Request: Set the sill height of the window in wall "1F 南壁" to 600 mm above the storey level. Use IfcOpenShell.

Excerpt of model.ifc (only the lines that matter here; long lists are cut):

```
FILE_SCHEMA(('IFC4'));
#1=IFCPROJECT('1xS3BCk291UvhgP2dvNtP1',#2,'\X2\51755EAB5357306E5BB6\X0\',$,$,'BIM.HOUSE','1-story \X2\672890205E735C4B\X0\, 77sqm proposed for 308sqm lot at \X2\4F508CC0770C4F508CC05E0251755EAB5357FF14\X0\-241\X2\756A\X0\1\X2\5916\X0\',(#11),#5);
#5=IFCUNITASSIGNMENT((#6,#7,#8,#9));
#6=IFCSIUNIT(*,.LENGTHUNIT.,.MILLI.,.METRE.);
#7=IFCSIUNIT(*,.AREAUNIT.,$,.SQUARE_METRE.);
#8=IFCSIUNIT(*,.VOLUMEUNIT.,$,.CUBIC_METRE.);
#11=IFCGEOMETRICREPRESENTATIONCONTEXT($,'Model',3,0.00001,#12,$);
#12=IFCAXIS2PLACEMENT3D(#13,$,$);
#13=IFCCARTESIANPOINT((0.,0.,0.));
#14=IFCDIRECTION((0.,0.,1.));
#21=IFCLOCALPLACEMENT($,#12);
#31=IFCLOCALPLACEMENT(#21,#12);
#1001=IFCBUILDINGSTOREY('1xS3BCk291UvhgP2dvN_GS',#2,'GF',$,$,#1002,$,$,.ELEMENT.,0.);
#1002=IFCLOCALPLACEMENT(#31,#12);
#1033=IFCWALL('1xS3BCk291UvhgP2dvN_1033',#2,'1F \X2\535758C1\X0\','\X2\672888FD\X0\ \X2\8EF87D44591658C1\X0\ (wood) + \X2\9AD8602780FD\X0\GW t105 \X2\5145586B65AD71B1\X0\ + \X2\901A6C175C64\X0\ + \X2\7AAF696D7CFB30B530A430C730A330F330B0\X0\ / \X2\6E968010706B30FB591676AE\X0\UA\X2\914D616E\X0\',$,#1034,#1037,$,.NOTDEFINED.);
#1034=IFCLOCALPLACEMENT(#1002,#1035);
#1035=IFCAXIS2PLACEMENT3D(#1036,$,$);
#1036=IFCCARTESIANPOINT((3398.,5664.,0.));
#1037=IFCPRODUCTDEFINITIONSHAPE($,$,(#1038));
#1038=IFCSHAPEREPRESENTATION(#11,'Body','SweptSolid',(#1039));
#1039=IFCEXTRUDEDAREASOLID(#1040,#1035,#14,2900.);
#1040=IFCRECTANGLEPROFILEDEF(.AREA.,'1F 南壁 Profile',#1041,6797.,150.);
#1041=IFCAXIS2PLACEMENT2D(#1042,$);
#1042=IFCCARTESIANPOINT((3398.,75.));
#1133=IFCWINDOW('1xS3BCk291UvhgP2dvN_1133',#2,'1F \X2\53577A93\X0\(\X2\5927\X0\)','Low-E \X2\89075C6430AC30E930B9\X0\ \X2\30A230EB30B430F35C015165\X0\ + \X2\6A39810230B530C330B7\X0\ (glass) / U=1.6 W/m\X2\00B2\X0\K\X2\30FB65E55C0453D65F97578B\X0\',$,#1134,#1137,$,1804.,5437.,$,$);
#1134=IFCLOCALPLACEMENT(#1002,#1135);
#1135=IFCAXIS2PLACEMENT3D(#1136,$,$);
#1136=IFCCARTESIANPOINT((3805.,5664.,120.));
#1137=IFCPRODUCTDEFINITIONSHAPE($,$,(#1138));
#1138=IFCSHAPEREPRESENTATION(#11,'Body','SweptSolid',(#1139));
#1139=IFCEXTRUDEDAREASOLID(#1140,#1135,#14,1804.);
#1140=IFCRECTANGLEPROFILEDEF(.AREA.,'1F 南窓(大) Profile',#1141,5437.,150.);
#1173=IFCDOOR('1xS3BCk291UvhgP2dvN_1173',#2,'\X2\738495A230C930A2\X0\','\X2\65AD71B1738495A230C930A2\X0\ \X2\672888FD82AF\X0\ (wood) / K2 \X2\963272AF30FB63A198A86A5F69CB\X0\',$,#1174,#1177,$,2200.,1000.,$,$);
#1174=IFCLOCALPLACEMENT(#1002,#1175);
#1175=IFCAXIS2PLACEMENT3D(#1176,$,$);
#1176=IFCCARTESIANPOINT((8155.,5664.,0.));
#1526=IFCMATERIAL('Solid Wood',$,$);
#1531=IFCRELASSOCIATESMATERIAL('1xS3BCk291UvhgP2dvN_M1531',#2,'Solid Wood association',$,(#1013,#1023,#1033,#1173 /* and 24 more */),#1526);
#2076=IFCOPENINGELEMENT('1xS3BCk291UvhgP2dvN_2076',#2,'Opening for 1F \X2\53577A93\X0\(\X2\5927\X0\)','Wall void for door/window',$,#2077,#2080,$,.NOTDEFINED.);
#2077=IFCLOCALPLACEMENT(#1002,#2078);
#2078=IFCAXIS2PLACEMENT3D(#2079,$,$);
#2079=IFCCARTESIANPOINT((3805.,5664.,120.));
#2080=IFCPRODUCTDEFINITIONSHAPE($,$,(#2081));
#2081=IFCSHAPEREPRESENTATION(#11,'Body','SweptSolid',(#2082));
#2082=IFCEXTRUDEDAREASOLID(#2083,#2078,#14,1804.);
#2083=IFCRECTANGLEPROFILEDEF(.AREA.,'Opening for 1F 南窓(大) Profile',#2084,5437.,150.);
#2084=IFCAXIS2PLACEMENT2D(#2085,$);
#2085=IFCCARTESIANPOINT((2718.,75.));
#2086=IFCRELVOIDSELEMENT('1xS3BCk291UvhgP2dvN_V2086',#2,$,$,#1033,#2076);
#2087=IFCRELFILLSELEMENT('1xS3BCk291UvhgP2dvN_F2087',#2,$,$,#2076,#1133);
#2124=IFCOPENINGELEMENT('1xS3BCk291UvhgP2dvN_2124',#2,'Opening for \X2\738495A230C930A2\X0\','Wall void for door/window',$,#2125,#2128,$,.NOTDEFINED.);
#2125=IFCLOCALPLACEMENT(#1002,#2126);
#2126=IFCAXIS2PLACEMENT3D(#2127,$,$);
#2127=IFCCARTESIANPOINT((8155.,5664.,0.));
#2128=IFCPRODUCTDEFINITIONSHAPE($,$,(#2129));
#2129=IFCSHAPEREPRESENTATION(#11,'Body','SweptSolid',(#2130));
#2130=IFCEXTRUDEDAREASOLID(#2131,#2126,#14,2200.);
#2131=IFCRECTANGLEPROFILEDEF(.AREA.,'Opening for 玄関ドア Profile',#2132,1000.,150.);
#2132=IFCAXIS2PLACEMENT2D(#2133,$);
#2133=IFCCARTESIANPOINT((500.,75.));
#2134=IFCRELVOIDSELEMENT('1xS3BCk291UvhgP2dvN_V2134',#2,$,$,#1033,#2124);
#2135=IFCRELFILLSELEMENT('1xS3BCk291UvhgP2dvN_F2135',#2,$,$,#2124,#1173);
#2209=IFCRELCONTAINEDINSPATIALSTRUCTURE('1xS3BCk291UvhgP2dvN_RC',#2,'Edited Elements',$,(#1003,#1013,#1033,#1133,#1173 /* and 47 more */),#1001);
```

```python
import numpy as np
import ifcopenshell
import ifcopenshell.api.geometry
import ifcopenshell.geom
import ifcopenshell.util.element
import ifcopenshell.util.placement
import ifcopenshell.util.shape
import ifcopenshell.util.unit

model = ifcopenshell.open("model.ifc")
unit_scale = ifcopenshell.util.unit.calculate_unit_scale(model)

window = model.by_guid("1xS3BCk291UvhgP2dvN_1133")
opening = window.FillsVoids[0].RelatingOpeningElement
storey = ifcopenshell.util.element.get_container(window, ifc_class="IfcBuildingStorey")
level = ifcopenshell.util.placement.get_local_placement(storey.ObjectPlacement)[2, 3]

# The opening's origin need not be at the sill, so measure its lowest point.
shape = ifcopenshell.geom.create_shape(ifcopenshell.geom.settings(), opening)
bottom = ifcopenshell.util.shape.get_shape_bottom_elevation(shape, shape.geometry) / unit_scale
dz = level + 600.0 - bottom

shift = np.array([0.0, 0.0, dz])
# The window is not placed relative to its opening, so move both.
for product in (opening, window):
    matrix = ifcopenshell.util.placement.get_local_placement(product.ObjectPlacement)
    matrix[:3, 3] += shift
    ifcopenshell.api.geometry.edit_object_placement(model, product=product, matrix=matrix, is_si=False)

print(f"moved by {dz * unit_scale:+.3f} m")

model.write("model_updated.ifc")
```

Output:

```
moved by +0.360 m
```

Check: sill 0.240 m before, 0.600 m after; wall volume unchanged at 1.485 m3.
